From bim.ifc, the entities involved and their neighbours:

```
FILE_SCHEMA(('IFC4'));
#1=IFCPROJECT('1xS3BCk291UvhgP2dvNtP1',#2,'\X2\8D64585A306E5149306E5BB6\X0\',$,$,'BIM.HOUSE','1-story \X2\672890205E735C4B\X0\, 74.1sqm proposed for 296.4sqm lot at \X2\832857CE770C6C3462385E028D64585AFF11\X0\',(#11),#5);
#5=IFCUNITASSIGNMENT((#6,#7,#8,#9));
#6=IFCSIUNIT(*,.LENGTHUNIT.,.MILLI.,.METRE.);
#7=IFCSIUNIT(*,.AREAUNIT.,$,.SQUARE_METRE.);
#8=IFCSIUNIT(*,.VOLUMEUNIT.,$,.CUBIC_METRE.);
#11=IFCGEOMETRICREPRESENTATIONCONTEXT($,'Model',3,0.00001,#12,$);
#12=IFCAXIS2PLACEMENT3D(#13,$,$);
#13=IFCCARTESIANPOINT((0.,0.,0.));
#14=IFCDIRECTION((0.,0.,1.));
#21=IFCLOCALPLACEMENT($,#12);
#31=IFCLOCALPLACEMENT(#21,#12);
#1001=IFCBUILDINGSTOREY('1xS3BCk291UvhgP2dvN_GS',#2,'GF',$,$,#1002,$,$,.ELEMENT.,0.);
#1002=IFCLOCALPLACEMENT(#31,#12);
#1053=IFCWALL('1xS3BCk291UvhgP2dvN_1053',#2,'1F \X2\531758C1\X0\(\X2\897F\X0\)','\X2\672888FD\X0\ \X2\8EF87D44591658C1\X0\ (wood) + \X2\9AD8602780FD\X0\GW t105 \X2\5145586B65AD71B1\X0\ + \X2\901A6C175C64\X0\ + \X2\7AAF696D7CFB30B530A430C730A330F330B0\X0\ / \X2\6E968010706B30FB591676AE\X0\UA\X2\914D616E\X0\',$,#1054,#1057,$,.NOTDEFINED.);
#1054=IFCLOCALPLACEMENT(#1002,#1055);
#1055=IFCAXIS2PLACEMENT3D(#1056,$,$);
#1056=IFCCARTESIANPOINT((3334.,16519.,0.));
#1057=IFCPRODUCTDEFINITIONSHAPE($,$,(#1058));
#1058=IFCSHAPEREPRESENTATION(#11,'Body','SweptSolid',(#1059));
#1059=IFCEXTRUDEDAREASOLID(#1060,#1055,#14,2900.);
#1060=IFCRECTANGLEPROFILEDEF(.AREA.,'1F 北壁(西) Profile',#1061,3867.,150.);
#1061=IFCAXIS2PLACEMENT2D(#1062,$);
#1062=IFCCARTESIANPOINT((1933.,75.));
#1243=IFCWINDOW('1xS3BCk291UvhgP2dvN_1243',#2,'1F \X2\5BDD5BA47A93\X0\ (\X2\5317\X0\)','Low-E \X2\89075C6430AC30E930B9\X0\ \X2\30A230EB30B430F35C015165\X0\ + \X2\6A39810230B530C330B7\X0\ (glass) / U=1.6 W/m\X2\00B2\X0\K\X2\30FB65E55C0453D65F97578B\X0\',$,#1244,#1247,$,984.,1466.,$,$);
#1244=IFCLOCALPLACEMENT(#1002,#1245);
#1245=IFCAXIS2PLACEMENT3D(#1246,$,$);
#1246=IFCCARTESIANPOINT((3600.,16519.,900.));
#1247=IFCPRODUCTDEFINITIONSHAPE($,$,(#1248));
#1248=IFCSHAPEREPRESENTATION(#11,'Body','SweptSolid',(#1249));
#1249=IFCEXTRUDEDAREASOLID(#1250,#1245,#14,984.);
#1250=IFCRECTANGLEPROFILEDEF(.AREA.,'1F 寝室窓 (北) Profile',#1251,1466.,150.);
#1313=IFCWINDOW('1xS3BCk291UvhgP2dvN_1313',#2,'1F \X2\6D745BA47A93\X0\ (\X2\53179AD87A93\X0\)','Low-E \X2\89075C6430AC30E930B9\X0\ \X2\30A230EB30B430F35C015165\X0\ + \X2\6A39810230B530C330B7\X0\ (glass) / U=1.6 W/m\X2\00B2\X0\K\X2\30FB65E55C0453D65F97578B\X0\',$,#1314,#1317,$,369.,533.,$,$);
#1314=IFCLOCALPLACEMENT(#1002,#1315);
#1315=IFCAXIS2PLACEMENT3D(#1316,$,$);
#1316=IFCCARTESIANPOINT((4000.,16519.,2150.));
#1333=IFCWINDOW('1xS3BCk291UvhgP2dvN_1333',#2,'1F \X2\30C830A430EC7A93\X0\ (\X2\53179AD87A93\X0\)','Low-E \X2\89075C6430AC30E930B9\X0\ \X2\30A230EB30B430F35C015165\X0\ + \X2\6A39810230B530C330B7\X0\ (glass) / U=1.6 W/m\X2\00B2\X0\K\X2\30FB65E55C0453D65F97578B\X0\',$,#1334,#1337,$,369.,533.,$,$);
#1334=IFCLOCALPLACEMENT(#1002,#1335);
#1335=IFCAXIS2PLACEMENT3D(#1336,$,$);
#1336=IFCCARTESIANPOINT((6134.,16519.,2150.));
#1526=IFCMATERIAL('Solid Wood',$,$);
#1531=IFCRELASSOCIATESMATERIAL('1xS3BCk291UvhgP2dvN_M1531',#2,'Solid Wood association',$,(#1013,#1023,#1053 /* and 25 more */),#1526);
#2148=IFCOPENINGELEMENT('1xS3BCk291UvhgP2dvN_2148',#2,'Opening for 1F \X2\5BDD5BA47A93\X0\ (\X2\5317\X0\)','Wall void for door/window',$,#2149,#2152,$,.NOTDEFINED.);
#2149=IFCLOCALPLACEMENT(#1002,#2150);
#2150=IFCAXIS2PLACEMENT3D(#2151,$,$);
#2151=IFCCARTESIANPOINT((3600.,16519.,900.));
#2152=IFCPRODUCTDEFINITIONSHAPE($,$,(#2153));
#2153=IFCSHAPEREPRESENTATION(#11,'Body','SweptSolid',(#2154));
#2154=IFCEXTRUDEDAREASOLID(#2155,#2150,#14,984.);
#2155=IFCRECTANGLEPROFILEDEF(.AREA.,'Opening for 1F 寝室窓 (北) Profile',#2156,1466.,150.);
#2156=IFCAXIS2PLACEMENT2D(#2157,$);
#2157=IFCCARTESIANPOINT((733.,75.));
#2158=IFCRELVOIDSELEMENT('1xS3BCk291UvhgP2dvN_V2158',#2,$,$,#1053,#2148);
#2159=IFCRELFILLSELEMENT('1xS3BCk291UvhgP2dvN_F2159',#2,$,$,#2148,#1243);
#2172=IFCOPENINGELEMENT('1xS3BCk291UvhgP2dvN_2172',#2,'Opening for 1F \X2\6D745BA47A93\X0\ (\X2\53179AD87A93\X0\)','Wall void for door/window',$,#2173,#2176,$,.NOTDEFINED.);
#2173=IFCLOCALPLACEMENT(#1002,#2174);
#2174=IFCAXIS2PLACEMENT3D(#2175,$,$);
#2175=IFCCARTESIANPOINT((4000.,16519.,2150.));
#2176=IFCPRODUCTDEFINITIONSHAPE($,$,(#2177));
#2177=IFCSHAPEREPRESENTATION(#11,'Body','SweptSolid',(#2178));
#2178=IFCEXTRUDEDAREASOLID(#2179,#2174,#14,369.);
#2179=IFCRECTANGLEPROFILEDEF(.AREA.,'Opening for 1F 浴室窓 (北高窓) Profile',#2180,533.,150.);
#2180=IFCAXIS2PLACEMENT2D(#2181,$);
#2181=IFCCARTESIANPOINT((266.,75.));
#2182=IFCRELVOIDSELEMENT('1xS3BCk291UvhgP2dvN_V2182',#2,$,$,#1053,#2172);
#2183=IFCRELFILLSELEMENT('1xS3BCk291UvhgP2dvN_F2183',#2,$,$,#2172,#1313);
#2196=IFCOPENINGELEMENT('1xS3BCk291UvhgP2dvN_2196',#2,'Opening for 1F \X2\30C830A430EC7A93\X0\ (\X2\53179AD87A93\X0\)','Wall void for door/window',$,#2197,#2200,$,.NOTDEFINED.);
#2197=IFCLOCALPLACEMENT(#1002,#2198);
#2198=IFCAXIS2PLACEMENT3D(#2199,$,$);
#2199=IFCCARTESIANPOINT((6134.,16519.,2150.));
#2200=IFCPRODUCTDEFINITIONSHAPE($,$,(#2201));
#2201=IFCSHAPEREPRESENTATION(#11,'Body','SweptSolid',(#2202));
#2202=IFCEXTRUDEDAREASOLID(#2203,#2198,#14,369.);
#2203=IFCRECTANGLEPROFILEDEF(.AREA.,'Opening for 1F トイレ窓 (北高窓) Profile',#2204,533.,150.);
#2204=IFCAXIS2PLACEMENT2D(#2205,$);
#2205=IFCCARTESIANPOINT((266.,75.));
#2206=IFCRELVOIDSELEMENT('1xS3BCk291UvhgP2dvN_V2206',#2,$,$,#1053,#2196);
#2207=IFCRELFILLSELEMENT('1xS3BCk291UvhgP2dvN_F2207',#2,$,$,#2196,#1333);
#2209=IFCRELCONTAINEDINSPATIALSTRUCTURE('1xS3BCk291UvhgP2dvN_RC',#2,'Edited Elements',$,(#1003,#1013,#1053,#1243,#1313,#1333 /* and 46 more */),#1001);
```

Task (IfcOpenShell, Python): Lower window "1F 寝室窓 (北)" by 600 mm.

```python
import numpy as np
import ifcopenshell
import ifcopenshell.api.geometry
import ifcopenshell.util.placement
import ifcopenshell.util.unit

model = ifcopenshell.open("bim.ifc")
unit_scale = ifcopenshell.util.unit.calculate_unit_scale(model)

window = model.by_guid("1xS3BCk291UvhgP2dvN_1243")
opening = window.FillsVoids[0].RelatingOpeningElement
dz = -0.6 / unit_scale

shift = np.array([0.0, 0.0, dz])
# The window is not placed relative to its opening, so move both.
for product in (opening, window):
    matrix = ifcopenshell.util.placement.get_local_placement(product.ObjectPlacement)
    matrix[:3, 3] += shift
    ifcopenshell.api.geometry.edit_object_placement(model, product=product, matrix=matrix, is_si=False)

print(f"moved by {dz * unit_scale:+.3f} m")

model.write("bim_v2.ifc")
```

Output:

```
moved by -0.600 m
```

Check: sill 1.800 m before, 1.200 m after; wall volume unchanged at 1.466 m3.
